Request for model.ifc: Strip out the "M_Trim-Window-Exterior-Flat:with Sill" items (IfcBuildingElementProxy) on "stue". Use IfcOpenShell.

First a look at what the model holds.

```python
import ifcopenshell
import ifcopenshell.util.element

model = ifcopenshell.open("model.ifc")
print(model.schema)
storey = next(s for s in model.by_type("IfcBuildingStorey") if s.Name == "stue")
proxies = [e for e in ifcopenshell.util.element.get_decomposition(storey) if e.is_a("IfcBuildingElementProxy")]
seen = {}
for e in proxies:
    element_type = ifcopenshell.util.element.get_type(e)
    name = element_type.Name if element_type not in (None, e) else None
    seen[name] = seen.get(name, 0) + 1
for name, count in sorted(seen.items(), key=str):
    print(count, "x", name)
```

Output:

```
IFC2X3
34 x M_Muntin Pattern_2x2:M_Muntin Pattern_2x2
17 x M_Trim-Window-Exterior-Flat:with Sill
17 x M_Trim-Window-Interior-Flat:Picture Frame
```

```python
import ifcopenshell
import ifcopenshell.api.root
import ifcopenshell.util.element

model = ifcopenshell.open("model.ifc")

storey = next(s for s in model.by_type("IfcBuildingStorey") if s.Name == "stue")
proxies = [e for e in ifcopenshell.util.element.get_decomposition(storey) if e.is_a("IfcBuildingElementProxy")]
targets = [e for e in proxies if (t := ifcopenshell.util.element.get_type(e)) not in (None, e) and t.Name == "M_Trim-Window-Exterior-Flat:with Sill"]

for e in targets:
    ifcopenshell.api.root.remove_product(model, product=e)
print(len(targets), "removed")

model.write("model-out.ifc")
```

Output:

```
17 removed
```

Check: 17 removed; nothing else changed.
